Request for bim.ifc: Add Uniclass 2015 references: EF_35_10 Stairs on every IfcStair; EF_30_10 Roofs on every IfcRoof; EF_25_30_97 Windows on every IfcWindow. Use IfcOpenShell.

First a look at what the model holds.

```python
import ifcopenshell

model = ifcopenshell.open("bim.ifc")
print(model.schema)
print("classifications:", [c.Name for c in model.by_type("IfcClassification")])
for ifc_class in ("IfcDoor", "IfcRoof", "IfcStair", "IfcWall", "IfcWindow"):
    print(ifc_class, len(model.by_type(ifc_class)))
```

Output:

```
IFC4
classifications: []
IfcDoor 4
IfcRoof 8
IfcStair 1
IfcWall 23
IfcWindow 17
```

```python
import ifcopenshell
import ifcopenshell.api.classification

model = ifcopenshell.open("bim.ifc")

system = ifcopenshell.api.classification.add_classification(model, classification="Uniclass 2015")

codes = {
    "IfcStair": ("EF_35_10", "Stairs"),
    "IfcRoof": ("EF_30_10", "Roofs"),
    "IfcWindow": ("EF_25_30_97", "Windows"),
}
for ifc_class, (code, name) in codes.items():
    products = model.by_type(ifc_class)
    ifcopenshell.api.classification.add_reference(
        model, products=products, classification=system, identification=code, name=name
    )
    print(code, len(products))

model.write("bim_edited.ifc")
```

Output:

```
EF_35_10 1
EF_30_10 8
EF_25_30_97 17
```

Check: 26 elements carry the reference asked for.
